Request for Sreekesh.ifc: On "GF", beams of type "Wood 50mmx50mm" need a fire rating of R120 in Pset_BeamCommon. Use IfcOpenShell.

First a look at what the model holds.

```python
import ifcopenshell
import ifcopenshell.util.element

model = ifcopenshell.open("Sreekesh.ifc")
print(model.schema)
storey = next(s for s in model.by_type("IfcBuildingStorey") if s.Name == "GF")
beams = [e for e in ifcopenshell.util.element.get_decomposition(storey) if e.is_a("IfcBeam")]
seen = {}
for e in beams:
    element_type = ifcopenshell.util.element.get_type(e)
    key = (element_type.Name if element_type != e and element_type else None, ifcopenshell.util.element.get_pset(e, "Pset_BeamCommon", "FireRating"))
    seen[key] = seen.get(key, 0) + 1
for (name, value), count in sorted(seen.items(), key=str):
    print(count, "x", name, "|", value)
```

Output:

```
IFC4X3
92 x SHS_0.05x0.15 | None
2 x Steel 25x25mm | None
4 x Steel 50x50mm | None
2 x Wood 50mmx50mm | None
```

```python
import ifcopenshell
import ifcopenshell.api.pset
import ifcopenshell.util.element

model = ifcopenshell.open("Sreekesh.ifc")

storey = next(s for s in model.by_type("IfcBuildingStorey") if s.Name == "GF")
beams = [e for e in ifcopenshell.util.element.get_decomposition(storey) if e.is_a("IfcBeam")]

count = 0
for e in beams:
    element_type = ifcopenshell.util.element.get_type(e)
    if element_type in (None, e) or element_type.Name != "Wood 50mmx50mm":
        continue
    # add_pset returns the element's existing set when there is one.
    pset = ifcopenshell.api.pset.add_pset(model, product=e, name="Pset_BeamCommon")
    ifcopenshell.api.pset.edit_pset(model, pset=pset, properties={"FireRating": "R120"})
    count += 1

print(count, "beams updated")

model.write("Sreekesh_rev.ifc")
```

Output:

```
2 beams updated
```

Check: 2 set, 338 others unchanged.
